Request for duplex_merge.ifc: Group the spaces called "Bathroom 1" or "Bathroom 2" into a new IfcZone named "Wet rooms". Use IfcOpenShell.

First a look at what the model holds.

```python
import ifcopenshell

model = ifcopenshell.open("duplex_merge.ifc")
print(model.schema)
seen = {}
for space in model.by_type("IfcSpace"):
    seen[space.LongName] = seen.get(space.LongName, 0) + 1
for name, count in sorted(seen.items(), key=str):
    print(count, "x", name)
print("zones:", [z.Name for z in model.by_type("IfcZone")][:20])
```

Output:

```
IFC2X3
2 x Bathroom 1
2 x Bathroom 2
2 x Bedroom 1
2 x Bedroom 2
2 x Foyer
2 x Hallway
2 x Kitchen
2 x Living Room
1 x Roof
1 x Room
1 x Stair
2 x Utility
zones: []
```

```python
import ifcopenshell
import ifcopenshell.api.group
import ifcopenshell.api.root

model = ifcopenshell.open("duplex_merge.ifc")

names = {"Bathroom 1", "Bathroom 2"}
spaces = [s for s in model.by_type("IfcSpace") if s.LongName in names]

zone = ifcopenshell.api.root.create_entity(model, ifc_class="IfcZone", name="Wet rooms")
ifcopenshell.api.group.assign_group(model, products=spaces, group=zone)
print(len(spaces), "spaces in", zone.Name)

model.write("duplex_merge_updated.ifc")
```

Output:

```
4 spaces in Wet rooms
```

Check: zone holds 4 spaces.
